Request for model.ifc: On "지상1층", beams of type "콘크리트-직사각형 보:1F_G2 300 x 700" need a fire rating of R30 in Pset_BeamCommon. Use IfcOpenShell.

First a look at what the model holds.

```python
import ifcopenshell
import ifcopenshell.util.element

model = ifcopenshell.open("model.ifc")
print(model.schema)
storey = next(s for s in model.by_type("IfcBuildingStorey") if s.Name == "지상1층")
beams = [e for e in ifcopenshell.util.element.get_decomposition(storey) if e.is_a("IfcBeam")]
seen = {}
for e in beams:
    element_type = ifcopenshell.util.element.get_type(e)
    key = (element_type.Name if element_type != e and element_type else None, ifcopenshell.util.element.get_pset(e, "Pset_BeamCommon", "FireRating"))
    seen[key] = seen.get(key, 0) + 1
for (name, value), count in sorted(seen.items(), key=str):
    print(count, "x", name, "|", value)
```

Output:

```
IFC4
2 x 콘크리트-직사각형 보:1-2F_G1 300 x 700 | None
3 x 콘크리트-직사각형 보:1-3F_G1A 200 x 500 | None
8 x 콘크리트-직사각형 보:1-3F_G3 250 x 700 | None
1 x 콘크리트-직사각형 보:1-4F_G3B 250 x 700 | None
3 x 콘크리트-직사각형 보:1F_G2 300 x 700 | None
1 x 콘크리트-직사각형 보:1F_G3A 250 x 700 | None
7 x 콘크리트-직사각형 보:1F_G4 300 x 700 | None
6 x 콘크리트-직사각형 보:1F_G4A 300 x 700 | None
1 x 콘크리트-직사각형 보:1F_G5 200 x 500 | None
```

```python
import ifcopenshell
import ifcopenshell.api.pset
import ifcopenshell.util.element

model = ifcopenshell.open("model.ifc")

storey = next(s for s in model.by_type("IfcBuildingStorey") if s.Name == "지상1층")
beams = [e for e in ifcopenshell.util.element.get_decomposition(storey) if e.is_a("IfcBeam")]

count = 0
for e in beams:
    element_type = ifcopenshell.util.element.get_type(e)
    if element_type in (None, e) or element_type.Name != "콘크리트-직사각형 보:1F_G2 300 x 700":
        continue
    # add_pset returns the element's existing set when there is one.
    pset = ifcopenshell.api.pset.add_pset(model, product=e, name="Pset_BeamCommon")
    ifcopenshell.api.pset.edit_pset(model, pset=pset, properties={"FireRating": "R30"})
    count += 1

print(count, "beams updated")

model.write("model_updated.ifc")
```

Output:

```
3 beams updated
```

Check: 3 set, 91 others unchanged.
